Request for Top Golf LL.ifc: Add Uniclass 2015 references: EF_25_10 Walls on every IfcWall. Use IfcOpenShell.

First a look at what the model holds.

```python
import ifcopenshell

model = ifcopenshell.open("Top Golf LL.ifc")
print(model.schema)
print("classifications:", [c.Name for c in model.by_type("IfcClassification")])
for ifc_class in ("IfcDoor", "IfcRoof", "IfcStair", "IfcWall", "IfcWindow"):
    print(ifc_class, len(model.by_type(ifc_class)))
```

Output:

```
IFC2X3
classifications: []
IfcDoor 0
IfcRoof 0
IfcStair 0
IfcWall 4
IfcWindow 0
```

```python
import ifcopenshell
import ifcopenshell.api.classification

model = ifcopenshell.open("Top Golf LL.ifc")

# IFC2X3 requires Source and Edition and has no link from the project to the system.
system = model.create_entity("IfcClassification", Source="NBS", Edition="2015", Name="Uniclass 2015")

codes = {
    "IfcWall": ("EF_25_10", "Walls"),
}
for ifc_class, (code, name) in codes.items():
    products = model.by_type(ifc_class)
    ifcopenshell.api.classification.add_reference(
        model, products=products, classification=system, identification=code, name=name
    )
    print(code, len(products))

model.write("Top Golf LL-out.ifc")
```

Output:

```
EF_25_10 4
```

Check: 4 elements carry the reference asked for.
